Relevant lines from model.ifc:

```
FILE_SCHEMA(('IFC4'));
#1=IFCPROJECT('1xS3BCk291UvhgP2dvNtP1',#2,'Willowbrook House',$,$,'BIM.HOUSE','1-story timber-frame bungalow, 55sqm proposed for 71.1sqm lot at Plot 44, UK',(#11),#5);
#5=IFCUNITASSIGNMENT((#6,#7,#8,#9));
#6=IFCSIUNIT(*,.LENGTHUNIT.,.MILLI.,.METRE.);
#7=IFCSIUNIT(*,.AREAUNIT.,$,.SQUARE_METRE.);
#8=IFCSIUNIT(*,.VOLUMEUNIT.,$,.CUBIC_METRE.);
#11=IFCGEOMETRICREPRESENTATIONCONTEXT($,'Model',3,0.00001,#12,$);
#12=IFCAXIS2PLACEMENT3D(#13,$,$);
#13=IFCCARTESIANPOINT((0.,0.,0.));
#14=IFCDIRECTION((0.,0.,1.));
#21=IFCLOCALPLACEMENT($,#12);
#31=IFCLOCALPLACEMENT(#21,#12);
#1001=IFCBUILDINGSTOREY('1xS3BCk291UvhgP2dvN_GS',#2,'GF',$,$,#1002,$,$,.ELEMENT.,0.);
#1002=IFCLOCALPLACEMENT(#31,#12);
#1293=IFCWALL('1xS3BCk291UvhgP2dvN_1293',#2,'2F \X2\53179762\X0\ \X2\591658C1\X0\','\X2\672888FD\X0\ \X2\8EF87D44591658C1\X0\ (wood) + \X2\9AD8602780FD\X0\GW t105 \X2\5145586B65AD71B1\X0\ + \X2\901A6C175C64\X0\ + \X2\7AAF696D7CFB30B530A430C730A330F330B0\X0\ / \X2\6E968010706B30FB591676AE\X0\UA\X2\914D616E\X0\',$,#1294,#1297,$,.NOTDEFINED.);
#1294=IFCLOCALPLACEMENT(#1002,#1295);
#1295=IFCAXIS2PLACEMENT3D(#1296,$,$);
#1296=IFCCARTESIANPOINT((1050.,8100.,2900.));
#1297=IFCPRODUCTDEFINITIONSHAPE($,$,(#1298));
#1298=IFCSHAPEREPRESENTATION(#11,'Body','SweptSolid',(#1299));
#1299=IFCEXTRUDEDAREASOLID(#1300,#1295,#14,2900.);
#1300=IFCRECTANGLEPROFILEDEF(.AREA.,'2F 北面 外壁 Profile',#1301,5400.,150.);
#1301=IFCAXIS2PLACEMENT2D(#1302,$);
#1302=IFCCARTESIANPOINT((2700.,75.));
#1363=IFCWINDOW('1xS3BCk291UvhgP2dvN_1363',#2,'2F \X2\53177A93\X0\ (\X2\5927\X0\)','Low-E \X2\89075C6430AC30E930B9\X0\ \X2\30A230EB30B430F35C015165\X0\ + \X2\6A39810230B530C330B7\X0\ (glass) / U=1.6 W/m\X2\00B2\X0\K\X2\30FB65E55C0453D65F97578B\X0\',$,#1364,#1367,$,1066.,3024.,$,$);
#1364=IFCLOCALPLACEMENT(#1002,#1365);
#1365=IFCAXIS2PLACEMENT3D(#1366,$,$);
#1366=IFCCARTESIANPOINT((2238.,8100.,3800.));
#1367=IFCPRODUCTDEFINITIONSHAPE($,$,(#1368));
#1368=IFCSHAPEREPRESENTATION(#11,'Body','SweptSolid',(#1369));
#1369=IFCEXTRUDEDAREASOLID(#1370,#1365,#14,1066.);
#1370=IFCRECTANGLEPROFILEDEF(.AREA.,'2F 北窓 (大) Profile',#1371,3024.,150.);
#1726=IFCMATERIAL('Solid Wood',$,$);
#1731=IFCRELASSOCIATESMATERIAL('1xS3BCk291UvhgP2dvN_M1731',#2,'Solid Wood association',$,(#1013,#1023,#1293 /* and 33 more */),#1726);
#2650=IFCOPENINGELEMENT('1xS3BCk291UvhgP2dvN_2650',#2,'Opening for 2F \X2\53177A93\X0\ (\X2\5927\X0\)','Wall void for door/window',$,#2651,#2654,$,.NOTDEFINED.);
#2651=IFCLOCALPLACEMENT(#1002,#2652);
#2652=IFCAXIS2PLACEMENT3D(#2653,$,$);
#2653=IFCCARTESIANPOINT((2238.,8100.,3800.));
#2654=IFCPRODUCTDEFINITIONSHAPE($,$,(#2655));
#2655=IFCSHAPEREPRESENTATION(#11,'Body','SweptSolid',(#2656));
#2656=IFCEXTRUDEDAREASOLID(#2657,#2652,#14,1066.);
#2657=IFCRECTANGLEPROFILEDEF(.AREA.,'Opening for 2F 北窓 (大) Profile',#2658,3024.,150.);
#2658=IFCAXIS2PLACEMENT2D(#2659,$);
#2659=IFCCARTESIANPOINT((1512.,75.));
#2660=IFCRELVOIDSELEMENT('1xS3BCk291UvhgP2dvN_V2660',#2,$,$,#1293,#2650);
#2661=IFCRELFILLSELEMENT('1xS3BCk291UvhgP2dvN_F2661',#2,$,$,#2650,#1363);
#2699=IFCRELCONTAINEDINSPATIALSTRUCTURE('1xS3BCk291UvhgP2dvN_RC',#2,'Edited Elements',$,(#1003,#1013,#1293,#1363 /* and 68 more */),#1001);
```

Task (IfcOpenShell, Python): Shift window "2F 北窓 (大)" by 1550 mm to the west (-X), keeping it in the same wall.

```python
import ifcopenshell
import ifcopenshell.api.geometry
import ifcopenshell.util.placement

model = ifcopenshell.open("model.ifc")

window = model.by_guid("1xS3BCk291UvhgP2dvN_1363")
opening = window.FillsVoids[0].RelatingOpeningElement
wall = opening.VoidsElements[0].RelatingBuildingElement

wall_matrix = ifcopenshell.util.placement.get_local_placement(wall.ObjectPlacement)
shift = wall_matrix[:3, 0] * -1550.0
before = ifcopenshell.util.placement.get_local_placement(window.ObjectPlacement)[:3, 3].copy()

# The window is not placed relative to its opening, so move both.
for product in (opening, window):
    matrix = ifcopenshell.util.placement.get_local_placement(product.ObjectPlacement)
    matrix[:3, 3] += shift
    ifcopenshell.api.geometry.edit_object_placement(model, product=product, matrix=matrix, is_si=False)

after = ifcopenshell.util.placement.get_local_placement(window.ObjectPlacement)[:3, 3]
print("window moved by", (after - before).round(3) + 0.0)

model.write("model_v2.ifc")
```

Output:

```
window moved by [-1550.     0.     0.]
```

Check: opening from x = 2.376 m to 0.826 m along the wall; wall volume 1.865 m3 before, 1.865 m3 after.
